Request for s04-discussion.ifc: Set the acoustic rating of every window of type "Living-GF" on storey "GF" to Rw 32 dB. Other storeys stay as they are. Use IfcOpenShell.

First a look at what the model holds.

```python
import ifcopenshell
import ifcopenshell.util.element

model = ifcopenshell.open("s04-discussion.ifc")
print(model.schema)
storey = next(s for s in model.by_type("IfcBuildingStorey") if s.Name == "GF")
windows = [e for e in ifcopenshell.util.element.get_decomposition(storey) if e.is_a("IfcWindow")]
seen = {}
for e in windows:
    element_type = ifcopenshell.util.element.get_type(e)
    key = (element_type.Name if element_type != e and element_type else None, ifcopenshell.util.element.get_pset(e, "Pset_WindowCommon", "AcousticRating"))
    seen[key] = seen.get(key, 0) + 1
for (name, value), count in sorted(seen.items(), key=str):
    print(count, "x", name, "|", value)
```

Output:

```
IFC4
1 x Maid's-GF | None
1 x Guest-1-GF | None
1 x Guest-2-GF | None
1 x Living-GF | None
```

```python
import ifcopenshell
import ifcopenshell.api.pset
import ifcopenshell.util.element

model = ifcopenshell.open("s04-discussion.ifc")

storey = next(s for s in model.by_type("IfcBuildingStorey") if s.Name == "GF")
windows = [e for e in ifcopenshell.util.element.get_decomposition(storey) if e.is_a("IfcWindow")]

count = 0
for e in windows:
    element_type = ifcopenshell.util.element.get_type(e)
    if element_type in (None, e) or element_type.Name != "Living-GF":
        continue
    # add_pset returns the element's existing set when there is one.
    pset = ifcopenshell.api.pset.add_pset(model, product=e, name="Pset_WindowCommon")
    ifcopenshell.api.pset.edit_pset(model, pset=pset, properties={"AcousticRating": "Rw 32 dB"})
    count += 1

print(count, "windows updated")

model.write("s04-discussion_v2.ifc")
```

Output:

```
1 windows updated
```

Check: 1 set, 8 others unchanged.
